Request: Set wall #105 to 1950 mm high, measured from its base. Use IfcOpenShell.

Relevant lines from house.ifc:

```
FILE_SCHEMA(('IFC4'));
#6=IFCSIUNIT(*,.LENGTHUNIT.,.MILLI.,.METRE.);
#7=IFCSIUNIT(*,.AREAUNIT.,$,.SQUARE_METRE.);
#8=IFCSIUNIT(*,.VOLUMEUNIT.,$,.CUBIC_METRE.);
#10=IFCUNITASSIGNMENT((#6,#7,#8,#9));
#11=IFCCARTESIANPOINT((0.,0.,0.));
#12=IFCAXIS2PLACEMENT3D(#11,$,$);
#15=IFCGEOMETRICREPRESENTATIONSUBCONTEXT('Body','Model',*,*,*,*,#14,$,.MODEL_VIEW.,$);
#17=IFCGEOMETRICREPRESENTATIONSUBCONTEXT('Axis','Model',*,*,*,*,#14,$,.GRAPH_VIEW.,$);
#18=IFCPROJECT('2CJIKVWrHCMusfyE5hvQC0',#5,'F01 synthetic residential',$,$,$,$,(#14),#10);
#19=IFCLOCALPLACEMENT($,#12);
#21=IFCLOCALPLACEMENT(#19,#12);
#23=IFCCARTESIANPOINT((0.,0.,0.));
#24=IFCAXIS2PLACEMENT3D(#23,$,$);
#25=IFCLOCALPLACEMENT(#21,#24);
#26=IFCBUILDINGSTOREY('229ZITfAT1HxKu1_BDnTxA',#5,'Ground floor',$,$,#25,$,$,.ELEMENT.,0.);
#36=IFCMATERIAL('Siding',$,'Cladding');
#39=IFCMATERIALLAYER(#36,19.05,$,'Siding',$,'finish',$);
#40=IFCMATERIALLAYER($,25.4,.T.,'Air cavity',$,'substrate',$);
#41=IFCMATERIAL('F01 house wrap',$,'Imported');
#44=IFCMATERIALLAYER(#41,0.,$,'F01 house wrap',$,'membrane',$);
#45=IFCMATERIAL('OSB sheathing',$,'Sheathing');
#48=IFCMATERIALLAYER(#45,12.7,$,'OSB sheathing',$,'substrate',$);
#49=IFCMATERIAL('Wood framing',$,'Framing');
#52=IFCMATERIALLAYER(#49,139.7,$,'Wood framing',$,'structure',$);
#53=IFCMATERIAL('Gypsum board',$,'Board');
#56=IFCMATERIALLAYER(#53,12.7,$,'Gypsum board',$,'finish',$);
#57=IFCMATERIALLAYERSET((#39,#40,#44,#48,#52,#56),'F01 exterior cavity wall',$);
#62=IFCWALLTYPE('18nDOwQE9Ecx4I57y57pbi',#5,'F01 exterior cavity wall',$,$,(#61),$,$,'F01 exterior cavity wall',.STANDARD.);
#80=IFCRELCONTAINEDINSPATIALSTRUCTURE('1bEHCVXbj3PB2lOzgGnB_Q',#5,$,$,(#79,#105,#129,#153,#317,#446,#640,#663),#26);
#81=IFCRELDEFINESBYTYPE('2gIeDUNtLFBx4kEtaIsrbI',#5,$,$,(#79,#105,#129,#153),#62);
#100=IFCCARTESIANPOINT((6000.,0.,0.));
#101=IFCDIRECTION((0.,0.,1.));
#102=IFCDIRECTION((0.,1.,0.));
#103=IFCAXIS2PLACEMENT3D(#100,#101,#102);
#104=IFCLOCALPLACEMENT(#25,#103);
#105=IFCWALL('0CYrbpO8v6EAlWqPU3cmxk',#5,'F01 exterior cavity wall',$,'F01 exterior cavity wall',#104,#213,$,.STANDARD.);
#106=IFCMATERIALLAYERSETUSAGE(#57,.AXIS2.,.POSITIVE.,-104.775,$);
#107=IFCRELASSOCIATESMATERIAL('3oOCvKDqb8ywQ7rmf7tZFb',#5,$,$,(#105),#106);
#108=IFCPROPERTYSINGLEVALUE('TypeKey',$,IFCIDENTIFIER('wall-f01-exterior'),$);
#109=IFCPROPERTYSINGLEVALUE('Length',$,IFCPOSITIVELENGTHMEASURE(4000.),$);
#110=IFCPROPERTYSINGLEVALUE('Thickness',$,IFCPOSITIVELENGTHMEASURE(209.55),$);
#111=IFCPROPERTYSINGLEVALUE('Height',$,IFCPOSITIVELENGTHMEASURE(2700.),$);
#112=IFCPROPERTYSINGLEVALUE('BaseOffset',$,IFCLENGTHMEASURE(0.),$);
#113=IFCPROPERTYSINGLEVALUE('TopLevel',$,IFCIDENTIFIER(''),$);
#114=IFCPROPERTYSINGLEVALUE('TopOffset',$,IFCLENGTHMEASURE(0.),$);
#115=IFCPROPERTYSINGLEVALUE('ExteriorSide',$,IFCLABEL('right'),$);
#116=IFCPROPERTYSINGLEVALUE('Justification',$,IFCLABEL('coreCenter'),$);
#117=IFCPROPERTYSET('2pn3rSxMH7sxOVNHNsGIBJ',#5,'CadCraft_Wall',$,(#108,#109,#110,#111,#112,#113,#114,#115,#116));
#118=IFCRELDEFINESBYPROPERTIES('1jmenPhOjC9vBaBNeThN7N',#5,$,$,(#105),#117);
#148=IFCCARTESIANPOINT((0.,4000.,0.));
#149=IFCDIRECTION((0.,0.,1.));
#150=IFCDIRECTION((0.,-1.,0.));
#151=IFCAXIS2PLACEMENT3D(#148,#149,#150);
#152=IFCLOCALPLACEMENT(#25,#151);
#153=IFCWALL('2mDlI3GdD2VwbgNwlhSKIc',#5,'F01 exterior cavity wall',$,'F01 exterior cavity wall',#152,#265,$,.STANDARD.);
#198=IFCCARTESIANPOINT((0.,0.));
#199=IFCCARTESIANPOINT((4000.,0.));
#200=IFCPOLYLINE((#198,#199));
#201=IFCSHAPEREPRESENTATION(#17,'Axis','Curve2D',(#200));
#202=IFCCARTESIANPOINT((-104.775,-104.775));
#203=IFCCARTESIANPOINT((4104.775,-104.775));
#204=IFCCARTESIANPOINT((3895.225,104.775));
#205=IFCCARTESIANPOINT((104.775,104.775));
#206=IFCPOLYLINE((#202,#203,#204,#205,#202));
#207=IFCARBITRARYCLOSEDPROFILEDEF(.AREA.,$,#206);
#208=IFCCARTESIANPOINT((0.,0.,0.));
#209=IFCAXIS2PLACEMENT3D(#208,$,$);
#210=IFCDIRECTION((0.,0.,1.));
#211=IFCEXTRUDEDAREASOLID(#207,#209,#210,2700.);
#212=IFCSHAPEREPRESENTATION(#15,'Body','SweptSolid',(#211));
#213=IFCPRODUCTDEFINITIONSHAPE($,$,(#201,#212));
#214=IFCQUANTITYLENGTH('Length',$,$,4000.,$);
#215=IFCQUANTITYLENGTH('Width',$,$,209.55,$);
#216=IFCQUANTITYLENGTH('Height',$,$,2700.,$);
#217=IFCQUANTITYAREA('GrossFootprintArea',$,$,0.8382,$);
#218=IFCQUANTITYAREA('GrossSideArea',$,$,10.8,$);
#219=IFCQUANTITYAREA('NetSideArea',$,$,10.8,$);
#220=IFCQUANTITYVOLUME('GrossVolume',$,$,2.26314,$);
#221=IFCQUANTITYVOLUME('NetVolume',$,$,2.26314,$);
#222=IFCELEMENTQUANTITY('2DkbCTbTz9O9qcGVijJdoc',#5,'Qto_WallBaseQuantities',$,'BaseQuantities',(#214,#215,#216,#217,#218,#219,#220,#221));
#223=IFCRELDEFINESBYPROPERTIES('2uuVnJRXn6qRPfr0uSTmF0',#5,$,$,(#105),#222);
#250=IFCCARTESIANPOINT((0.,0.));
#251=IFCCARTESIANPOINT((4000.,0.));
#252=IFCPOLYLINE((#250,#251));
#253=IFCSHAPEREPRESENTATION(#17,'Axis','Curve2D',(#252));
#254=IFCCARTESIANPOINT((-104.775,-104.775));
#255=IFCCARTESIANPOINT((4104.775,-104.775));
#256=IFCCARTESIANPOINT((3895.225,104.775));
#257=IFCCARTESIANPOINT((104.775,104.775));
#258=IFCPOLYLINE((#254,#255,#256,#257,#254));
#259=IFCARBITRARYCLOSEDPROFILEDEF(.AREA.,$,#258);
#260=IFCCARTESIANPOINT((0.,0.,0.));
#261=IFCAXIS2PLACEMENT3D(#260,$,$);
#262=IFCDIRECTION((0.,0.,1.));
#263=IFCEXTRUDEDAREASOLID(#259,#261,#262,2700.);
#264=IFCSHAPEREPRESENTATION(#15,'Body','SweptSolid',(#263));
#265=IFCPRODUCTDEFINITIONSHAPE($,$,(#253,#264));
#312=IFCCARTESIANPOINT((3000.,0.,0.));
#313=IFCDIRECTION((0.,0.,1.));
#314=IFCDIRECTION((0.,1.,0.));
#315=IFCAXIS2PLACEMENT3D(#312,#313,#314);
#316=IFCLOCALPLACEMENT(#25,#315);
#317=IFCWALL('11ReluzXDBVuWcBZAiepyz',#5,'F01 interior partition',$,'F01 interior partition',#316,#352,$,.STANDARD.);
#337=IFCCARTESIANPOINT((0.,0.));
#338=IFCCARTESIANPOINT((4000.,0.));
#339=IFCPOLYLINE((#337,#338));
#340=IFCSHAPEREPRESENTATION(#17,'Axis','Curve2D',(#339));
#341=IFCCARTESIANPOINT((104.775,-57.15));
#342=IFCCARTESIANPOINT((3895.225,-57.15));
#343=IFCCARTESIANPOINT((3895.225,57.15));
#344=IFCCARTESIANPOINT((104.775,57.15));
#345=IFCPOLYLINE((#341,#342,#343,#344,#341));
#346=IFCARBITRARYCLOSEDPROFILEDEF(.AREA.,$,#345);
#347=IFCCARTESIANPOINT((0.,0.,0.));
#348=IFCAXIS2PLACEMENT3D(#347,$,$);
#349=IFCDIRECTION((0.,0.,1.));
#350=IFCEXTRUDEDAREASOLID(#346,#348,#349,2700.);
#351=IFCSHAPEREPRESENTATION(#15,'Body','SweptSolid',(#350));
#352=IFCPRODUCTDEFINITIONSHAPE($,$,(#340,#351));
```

```python
import ifcopenshell
import ifcopenshell.api.pset
import ifcopenshell.geom
import ifcopenshell.util.element
import ifcopenshell.util.representation
import ifcopenshell.util.shape
import ifcopenshell.util.unit

model = ifcopenshell.open("house.ifc")
unit_scale = ifcopenshell.util.unit.calculate_unit_scale(model)
area_scale = ifcopenshell.util.unit.calculate_unit_scale(model, "AREAUNIT")
volume_scale = ifcopenshell.util.unit.calculate_unit_scale(model, "VOLUMEUNIT")
settings = ifcopenshell.geom.settings()


def volume(element):
    """Net volume in cubic metres, openings subtracted."""
    shape = ifcopenshell.geom.create_shape(settings, element)
    return ifcopenshell.util.shape.get_volume(shape.geometry)


wall = model.by_guid("0CYrbpO8v6EAlWqPU3cmxk")
before = volume(wall)

body = ifcopenshell.util.representation.get_representation(wall, "Model", "Body")
solid = body.Items[0]
old_height = solid.Depth
solid.Depth = 1.95 / unit_scale
after = volume(wall)
thickness = 0.2096  # wall thickness in metres

# Update the stored height, areas and volumes.
pset = model.by_id(ifcopenshell.util.element.get_pset(wall, "CadCraft_Wall", should_inherit=False)["id"])
ifcopenshell.api.pset.edit_pset(model, pset=pset, properties={
    "Height": model.create_entity("IfcPositiveLengthMeasure", solid.Depth),
})
qto = model.by_id(ifcopenshell.util.element.get_pset(wall, "Qto_WallBaseQuantities", should_inherit=False)["id"])
ifcopenshell.api.pset.edit_qto(model, qto=qto, properties={
    "Height": solid.Depth,
    "GrossSideArea": ifcopenshell.util.element.get_pset(wall, "Qto_WallBaseQuantities", "GrossSideArea") * solid.Depth / old_height,
    "NetSideArea": after / thickness / area_scale,
    "GrossVolume": ifcopenshell.util.element.get_pset(wall, "Qto_WallBaseQuantities", "GrossVolume") * solid.Depth / old_height,
    "NetVolume": after / volume_scale,
})

print(f"height {old_height:g} -> {solid.Depth:g}, volume {before:.3f} -> {after:.3f} m3")

model.write("house_edited.ifc")
```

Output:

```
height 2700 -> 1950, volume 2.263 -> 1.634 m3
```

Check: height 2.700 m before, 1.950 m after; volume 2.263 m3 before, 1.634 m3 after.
